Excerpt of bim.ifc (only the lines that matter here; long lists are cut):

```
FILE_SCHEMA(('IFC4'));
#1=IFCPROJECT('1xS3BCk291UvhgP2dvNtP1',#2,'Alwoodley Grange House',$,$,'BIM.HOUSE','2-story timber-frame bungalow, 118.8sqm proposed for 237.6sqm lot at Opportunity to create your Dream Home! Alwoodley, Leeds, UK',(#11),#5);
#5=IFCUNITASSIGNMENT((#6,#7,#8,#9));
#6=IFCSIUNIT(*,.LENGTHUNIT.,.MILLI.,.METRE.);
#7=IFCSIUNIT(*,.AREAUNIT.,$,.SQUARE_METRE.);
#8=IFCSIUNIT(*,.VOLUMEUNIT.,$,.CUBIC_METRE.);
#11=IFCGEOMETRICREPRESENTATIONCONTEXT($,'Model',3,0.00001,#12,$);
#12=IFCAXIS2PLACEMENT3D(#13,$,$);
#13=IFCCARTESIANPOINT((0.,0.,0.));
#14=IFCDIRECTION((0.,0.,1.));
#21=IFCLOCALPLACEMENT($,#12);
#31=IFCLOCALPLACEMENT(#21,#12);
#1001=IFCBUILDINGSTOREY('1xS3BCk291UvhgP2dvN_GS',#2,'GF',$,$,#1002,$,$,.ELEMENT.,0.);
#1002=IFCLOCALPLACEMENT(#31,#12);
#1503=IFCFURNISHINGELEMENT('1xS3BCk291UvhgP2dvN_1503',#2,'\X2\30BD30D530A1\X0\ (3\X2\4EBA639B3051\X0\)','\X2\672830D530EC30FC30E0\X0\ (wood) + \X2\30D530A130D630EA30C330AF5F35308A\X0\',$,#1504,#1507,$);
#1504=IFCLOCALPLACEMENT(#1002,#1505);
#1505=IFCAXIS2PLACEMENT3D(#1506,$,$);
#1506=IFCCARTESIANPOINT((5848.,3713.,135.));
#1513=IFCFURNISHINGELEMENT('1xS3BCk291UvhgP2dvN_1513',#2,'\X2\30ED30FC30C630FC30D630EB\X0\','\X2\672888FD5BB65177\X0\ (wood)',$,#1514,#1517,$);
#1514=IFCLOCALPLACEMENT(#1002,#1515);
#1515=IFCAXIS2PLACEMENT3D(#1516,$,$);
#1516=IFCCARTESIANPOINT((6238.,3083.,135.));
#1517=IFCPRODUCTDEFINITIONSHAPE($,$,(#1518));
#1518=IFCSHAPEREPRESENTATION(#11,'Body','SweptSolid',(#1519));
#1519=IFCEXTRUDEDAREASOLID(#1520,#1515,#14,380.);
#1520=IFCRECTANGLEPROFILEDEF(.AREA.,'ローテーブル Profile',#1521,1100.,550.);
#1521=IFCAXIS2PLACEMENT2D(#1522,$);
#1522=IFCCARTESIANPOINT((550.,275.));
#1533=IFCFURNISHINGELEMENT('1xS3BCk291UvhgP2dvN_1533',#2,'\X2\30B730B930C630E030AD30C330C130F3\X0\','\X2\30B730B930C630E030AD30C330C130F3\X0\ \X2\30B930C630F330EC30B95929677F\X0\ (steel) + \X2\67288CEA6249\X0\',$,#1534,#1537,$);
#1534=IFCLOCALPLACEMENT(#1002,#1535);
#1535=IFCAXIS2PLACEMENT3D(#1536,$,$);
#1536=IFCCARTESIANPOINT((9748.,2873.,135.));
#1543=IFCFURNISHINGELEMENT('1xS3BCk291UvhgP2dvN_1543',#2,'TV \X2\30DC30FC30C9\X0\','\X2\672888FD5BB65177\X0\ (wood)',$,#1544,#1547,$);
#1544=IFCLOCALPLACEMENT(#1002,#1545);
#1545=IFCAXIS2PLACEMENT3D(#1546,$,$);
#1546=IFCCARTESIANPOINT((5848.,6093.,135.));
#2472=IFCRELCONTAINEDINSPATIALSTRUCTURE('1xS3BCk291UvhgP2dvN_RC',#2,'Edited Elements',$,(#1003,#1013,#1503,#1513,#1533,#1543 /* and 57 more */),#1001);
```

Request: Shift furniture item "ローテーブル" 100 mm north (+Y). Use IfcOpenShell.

```python
import ifcopenshell
import ifcopenshell.api.geometry
import ifcopenshell.util.placement
import ifcopenshell.util.unit

model = ifcopenshell.open("bim.ifc")
unit_scale = ifcopenshell.util.unit.calculate_unit_scale(model)

item = model.by_id(1513)
matrix = ifcopenshell.util.placement.get_local_placement(item.ObjectPlacement)
matrix[1, 3] += 0.1 / unit_scale
ifcopenshell.api.geometry.edit_object_placement(model, product=item, matrix=matrix, is_si=False)

print(ifcopenshell.util.placement.get_local_placement(item.ObjectPlacement).round(3) + 0.0)

model.write("bim_edited.ifc")
```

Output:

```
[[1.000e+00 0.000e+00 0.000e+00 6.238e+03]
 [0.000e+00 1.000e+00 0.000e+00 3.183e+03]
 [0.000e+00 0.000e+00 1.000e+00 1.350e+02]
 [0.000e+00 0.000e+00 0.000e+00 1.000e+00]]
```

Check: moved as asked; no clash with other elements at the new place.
